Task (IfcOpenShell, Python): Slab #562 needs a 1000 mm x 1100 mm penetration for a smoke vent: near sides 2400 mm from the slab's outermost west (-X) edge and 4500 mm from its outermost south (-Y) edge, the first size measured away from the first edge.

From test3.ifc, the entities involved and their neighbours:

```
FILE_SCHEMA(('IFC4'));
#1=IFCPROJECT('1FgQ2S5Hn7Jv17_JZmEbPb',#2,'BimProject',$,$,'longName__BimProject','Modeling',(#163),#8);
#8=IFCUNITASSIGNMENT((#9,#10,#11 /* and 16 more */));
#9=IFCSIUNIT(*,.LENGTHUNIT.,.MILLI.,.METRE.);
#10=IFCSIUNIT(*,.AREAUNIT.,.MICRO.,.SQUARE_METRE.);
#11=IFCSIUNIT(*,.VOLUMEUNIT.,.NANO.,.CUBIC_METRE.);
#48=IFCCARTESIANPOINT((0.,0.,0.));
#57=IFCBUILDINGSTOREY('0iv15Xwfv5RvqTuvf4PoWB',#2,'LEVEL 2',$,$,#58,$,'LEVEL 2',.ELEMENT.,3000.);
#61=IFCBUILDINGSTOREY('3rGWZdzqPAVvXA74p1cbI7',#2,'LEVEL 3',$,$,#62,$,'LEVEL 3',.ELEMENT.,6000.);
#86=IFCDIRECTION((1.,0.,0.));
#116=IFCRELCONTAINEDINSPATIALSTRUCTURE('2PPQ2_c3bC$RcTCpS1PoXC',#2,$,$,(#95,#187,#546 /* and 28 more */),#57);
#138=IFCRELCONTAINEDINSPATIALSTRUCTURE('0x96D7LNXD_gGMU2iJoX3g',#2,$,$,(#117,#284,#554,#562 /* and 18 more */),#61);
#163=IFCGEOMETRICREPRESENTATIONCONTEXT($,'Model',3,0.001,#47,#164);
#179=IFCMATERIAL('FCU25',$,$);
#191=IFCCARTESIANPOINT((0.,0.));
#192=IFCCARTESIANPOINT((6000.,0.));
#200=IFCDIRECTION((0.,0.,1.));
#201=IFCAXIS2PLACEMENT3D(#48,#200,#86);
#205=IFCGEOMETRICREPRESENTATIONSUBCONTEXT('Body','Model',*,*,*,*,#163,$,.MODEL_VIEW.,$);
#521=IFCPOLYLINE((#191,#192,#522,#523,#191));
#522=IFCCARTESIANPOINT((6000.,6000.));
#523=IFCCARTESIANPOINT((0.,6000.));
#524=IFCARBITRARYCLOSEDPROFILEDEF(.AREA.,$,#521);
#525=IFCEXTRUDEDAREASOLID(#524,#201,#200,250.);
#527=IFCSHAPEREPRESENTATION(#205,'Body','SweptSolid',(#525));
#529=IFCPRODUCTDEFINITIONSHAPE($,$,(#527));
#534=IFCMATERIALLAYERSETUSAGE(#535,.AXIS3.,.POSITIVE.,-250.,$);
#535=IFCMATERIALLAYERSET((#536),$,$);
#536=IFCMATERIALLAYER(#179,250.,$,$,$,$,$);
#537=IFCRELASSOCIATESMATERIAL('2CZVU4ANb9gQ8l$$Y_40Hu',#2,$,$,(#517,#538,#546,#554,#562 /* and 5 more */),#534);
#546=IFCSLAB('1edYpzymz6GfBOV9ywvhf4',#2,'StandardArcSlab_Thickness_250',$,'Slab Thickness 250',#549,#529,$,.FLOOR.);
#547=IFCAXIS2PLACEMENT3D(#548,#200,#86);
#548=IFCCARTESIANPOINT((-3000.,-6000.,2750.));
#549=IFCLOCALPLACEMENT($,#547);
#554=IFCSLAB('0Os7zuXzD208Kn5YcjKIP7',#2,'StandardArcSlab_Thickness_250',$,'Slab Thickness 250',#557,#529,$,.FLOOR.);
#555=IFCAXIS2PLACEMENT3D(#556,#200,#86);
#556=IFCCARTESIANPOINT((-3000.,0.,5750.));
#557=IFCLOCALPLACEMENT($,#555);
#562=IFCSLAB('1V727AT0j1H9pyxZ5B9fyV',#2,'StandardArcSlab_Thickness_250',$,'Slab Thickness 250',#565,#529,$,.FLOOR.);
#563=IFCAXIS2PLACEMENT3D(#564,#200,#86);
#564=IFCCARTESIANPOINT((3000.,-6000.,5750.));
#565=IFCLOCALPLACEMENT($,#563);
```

```python
import numpy as np
import ifcopenshell
import ifcopenshell.api.feature
import ifcopenshell.api.geometry
import ifcopenshell.api.root
import ifcopenshell.geom
import ifcopenshell.util.placement
import ifcopenshell.util.representation
import ifcopenshell.util.shape
import ifcopenshell.util.unit

model = ifcopenshell.open("test3.ifc")
unit_scale = ifcopenshell.util.unit.calculate_unit_scale(model)
settings = ifcopenshell.geom.settings()


def volume(element):
    """Net volume in cubic metres, openings subtracted."""
    shape = ifcopenshell.geom.create_shape(settings, element)
    return ifcopenshell.util.shape.get_volume(shape.geometry)


slab = model.by_guid("1V727AT0j1H9pyxZ5B9fyV")
before = volume(slab)

# Extent in the slab's own axes, in metres. The edges named are its -X and -Y sides.
slab_shape = ifcopenshell.geom.create_shape(settings, slab)
vertices = ifcopenshell.util.shape.get_vertices(slab_shape.geometry)
x_min, y_min, bottom = vertices.min(axis=0)
top = vertices[:, 2].max()

opening = ifcopenshell.api.root.create_entity(model, ifc_class="IfcOpeningElement", name="Smoke vent opening", predefined_type="OPENING")
context = ifcopenshell.util.representation.get_context(model, "Model", "Body", "MODEL_VIEW")
width, depth = 1, 1.1
outline = [(0.0, 0.0), (width, 0.0), (width, depth), (0.0, depth), (0.0, 0.0)]
# Overshoot both faces by 50 mm so the cut is clean.
shape = ifcopenshell.api.geometry.add_slab_representation(
    model, context=context, depth=top - bottom + 0.1, polyline=outline
)
ifcopenshell.api.geometry.assign_representation(model, product=opening, representation=shape)

matrix = ifcopenshell.util.placement.get_local_placement(slab.ObjectPlacement)
matrix[:, 3] = matrix @ np.append(np.array([x_min + 2.4, y_min + 4.5, bottom - 0.05]) / unit_scale, 1.0)
ifcopenshell.api.geometry.edit_object_placement(model, product=opening, matrix=matrix, is_si=False)
ifcopenshell.api.feature.add_feature(model, feature=opening, element=slab)

after = volume(slab)

print(f"slab volume {before:.3f} -> {after:.3f} m3")

model.write("test3_updated.ifc")
```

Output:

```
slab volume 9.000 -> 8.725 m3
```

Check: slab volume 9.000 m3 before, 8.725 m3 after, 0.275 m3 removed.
